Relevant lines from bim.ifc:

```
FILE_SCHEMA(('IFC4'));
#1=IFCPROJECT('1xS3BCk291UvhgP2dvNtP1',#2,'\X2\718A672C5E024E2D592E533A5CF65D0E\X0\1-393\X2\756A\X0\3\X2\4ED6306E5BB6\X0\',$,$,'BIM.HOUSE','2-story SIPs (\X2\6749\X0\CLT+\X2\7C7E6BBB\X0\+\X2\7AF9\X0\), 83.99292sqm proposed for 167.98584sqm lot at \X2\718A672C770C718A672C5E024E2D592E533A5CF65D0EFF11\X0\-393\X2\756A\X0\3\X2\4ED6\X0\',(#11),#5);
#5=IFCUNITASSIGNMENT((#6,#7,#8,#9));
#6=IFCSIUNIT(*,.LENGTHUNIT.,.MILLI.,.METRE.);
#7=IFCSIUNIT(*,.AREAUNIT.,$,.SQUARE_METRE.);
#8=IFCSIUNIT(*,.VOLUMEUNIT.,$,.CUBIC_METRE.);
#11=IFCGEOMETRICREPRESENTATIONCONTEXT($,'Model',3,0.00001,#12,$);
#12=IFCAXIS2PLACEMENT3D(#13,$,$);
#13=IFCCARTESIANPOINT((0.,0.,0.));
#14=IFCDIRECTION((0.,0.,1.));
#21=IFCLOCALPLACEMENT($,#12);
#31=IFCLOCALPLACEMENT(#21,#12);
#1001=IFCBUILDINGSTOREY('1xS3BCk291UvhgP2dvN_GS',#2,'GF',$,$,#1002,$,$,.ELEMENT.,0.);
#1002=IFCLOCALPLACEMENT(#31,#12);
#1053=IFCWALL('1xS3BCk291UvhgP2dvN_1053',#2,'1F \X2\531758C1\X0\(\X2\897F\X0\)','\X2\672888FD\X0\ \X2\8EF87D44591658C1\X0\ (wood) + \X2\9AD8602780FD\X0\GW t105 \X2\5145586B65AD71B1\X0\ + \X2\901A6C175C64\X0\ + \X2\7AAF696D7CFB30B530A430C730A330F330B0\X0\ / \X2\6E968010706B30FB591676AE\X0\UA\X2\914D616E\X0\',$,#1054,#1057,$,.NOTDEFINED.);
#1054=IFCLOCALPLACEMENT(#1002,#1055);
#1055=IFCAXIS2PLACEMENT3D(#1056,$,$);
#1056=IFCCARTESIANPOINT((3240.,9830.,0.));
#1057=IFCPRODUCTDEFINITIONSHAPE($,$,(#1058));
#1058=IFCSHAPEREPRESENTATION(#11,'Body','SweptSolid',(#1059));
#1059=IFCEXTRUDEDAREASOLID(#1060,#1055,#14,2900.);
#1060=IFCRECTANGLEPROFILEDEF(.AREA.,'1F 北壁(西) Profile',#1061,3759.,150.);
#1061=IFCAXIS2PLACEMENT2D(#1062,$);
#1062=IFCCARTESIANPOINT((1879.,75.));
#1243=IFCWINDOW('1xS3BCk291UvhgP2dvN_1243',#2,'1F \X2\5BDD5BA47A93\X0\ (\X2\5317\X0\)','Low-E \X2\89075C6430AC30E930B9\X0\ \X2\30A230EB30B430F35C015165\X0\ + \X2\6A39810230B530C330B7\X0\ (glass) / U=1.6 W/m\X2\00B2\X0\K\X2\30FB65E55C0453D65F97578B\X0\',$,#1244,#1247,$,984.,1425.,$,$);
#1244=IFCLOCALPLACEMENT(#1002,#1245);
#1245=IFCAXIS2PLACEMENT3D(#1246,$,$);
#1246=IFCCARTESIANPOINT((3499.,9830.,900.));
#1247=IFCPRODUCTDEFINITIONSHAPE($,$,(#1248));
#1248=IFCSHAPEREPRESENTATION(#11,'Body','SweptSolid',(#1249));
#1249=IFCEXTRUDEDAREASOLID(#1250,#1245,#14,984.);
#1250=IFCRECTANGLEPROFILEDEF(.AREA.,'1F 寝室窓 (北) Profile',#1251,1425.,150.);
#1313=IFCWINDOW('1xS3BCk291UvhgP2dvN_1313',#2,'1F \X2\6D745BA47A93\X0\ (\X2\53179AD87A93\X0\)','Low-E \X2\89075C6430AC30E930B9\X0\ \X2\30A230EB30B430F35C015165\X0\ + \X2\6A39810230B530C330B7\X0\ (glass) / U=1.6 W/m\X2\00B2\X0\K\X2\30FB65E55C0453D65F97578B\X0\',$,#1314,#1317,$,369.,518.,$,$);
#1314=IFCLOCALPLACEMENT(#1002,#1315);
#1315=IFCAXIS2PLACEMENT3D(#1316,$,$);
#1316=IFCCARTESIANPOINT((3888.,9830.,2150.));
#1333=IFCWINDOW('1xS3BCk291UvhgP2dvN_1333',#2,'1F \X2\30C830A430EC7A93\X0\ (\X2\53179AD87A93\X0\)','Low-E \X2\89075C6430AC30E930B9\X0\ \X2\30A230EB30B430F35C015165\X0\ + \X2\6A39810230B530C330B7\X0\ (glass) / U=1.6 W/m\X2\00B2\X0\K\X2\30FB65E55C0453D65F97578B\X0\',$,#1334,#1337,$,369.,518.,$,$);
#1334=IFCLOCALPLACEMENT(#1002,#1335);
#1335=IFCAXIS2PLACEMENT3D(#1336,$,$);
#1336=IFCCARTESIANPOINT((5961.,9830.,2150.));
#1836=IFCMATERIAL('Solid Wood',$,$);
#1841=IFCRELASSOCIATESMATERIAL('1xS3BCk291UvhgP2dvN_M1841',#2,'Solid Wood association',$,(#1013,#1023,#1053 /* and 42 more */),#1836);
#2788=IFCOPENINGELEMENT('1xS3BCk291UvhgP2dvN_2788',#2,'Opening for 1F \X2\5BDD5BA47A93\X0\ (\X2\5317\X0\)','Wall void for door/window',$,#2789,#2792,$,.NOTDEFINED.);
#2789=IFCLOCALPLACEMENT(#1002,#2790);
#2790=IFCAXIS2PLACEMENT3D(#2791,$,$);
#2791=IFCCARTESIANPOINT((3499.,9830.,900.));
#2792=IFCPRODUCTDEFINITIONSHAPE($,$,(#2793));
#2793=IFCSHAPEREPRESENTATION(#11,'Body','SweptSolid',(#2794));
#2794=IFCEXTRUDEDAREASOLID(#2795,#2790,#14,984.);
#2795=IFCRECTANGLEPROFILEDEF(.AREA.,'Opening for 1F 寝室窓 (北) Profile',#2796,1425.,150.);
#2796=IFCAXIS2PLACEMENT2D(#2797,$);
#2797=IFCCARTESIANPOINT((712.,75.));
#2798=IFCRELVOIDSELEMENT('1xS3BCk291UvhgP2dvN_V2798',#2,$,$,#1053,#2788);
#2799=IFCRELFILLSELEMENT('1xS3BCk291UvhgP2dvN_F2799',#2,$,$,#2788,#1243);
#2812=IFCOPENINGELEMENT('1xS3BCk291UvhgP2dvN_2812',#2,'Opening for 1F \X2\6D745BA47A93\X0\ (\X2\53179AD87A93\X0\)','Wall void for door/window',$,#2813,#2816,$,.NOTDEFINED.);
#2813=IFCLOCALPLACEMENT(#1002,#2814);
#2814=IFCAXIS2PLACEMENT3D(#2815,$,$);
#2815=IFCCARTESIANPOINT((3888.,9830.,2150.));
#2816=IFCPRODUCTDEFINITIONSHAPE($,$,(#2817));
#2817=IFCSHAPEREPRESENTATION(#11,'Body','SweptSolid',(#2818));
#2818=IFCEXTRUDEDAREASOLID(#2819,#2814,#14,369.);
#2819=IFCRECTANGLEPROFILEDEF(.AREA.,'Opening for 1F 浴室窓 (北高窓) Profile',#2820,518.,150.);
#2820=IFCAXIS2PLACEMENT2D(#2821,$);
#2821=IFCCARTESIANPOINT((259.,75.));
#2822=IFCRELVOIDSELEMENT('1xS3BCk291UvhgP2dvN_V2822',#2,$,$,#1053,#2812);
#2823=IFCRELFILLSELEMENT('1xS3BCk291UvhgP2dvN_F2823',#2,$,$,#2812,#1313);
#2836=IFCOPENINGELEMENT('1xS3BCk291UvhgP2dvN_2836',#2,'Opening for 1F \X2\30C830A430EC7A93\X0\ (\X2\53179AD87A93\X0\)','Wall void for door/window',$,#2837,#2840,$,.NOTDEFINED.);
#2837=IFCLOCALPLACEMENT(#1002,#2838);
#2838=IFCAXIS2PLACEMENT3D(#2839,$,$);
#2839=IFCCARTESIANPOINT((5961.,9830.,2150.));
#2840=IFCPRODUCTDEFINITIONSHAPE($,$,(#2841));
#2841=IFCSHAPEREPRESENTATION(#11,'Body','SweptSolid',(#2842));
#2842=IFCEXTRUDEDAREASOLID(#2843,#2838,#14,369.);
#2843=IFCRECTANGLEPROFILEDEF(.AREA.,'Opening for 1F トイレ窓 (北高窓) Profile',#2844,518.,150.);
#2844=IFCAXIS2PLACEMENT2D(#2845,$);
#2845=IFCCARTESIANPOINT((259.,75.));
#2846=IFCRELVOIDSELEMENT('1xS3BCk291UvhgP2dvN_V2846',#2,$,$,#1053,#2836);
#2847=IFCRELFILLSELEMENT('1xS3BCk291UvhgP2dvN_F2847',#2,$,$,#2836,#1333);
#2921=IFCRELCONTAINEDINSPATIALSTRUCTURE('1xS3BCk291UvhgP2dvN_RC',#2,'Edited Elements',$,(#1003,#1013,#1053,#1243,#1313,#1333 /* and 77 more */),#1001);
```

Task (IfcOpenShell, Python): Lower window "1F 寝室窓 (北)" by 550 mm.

```python
import numpy as np
import ifcopenshell
import ifcopenshell.api.geometry
import ifcopenshell.util.placement
import ifcopenshell.util.unit

model = ifcopenshell.open("bim.ifc")
unit_scale = ifcopenshell.util.unit.calculate_unit_scale(model)

window = model.by_id(1243)
opening = window.FillsVoids[0].RelatingOpeningElement
dz = -0.55 / unit_scale

shift = np.array([0.0, 0.0, dz])
# The window is not placed relative to its opening, so move both.
for product in (opening, window):
    matrix = ifcopenshell.util.placement.get_local_placement(product.ObjectPlacement)
    matrix[:3, 3] += shift
    ifcopenshell.api.geometry.edit_object_placement(model, product=product, matrix=matrix, is_si=False)

print(f"moved by {dz * unit_scale:+.3f} m")

model.write("bim_v2.ifc")
```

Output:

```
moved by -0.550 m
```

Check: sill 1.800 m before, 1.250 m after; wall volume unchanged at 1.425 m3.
